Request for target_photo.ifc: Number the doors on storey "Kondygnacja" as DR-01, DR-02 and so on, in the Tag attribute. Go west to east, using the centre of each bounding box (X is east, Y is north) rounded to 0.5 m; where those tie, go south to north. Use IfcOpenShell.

First a look at what the model holds.

```python
import ifcopenshell
import ifcopenshell.util.element
import ifcopenshell.util.placement

model = ifcopenshell.open("target_photo.ifc")
print(model.schema)
storey = next(s for s in model.by_type("IfcBuildingStorey") if s.Name == "Kondygnacja")
doors = [e for e in ifcopenshell.util.element.get_decomposition(storey) if e.is_a("IfcDoor")]
for e in sorted(doors, key=lambda e: e.id()):
    origin = ifcopenshell.util.placement.get_local_placement(e.ObjectPlacement)[:3, 3]
    print(e.id(), e.Tag, e.Name, origin.round(2) + 0.0, sep=" | ")
```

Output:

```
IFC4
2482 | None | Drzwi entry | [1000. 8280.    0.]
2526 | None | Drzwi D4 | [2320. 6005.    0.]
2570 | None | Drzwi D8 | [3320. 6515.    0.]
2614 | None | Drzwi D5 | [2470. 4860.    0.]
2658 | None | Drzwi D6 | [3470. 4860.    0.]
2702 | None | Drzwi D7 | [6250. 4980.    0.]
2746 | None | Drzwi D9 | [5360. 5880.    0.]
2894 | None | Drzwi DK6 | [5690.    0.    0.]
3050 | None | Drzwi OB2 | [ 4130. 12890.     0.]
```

```python
import ifcopenshell
import ifcopenshell.geom
import ifcopenshell.util.element
import ifcopenshell.util.shape

model = ifcopenshell.open("target_photo.ifc")
settings = ifcopenshell.geom.settings()
settings.set("use-world-coords", True)


def centre(element):
    shape = ifcopenshell.geom.create_shape(settings, element)
    return ifcopenshell.util.shape.get_bbox_centroid(shape.geometry)


storey = next(s for s in model.by_type("IfcBuildingStorey") if s.Name == "Kondygnacja")
doors = [e for e in ifcopenshell.util.element.get_decomposition(storey) if e.is_a("IfcDoor")]

# Insertion points can sit at a corner or the storey origin, so sort by the geometry (in metres).
centres = {e: centre(e) for e in doors}
doors.sort(key=lambda e: (round(centres[e][0] / 0.5), centres[e][1]))

for i, e in enumerate(doors, start=1):
    number = f"DR-{i:02d}"
    e.Tag = number
    print(e.id(), number)

model.write("target_photo_v2.ifc")
```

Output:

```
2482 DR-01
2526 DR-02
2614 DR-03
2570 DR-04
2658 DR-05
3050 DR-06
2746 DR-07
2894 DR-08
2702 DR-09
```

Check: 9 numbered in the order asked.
